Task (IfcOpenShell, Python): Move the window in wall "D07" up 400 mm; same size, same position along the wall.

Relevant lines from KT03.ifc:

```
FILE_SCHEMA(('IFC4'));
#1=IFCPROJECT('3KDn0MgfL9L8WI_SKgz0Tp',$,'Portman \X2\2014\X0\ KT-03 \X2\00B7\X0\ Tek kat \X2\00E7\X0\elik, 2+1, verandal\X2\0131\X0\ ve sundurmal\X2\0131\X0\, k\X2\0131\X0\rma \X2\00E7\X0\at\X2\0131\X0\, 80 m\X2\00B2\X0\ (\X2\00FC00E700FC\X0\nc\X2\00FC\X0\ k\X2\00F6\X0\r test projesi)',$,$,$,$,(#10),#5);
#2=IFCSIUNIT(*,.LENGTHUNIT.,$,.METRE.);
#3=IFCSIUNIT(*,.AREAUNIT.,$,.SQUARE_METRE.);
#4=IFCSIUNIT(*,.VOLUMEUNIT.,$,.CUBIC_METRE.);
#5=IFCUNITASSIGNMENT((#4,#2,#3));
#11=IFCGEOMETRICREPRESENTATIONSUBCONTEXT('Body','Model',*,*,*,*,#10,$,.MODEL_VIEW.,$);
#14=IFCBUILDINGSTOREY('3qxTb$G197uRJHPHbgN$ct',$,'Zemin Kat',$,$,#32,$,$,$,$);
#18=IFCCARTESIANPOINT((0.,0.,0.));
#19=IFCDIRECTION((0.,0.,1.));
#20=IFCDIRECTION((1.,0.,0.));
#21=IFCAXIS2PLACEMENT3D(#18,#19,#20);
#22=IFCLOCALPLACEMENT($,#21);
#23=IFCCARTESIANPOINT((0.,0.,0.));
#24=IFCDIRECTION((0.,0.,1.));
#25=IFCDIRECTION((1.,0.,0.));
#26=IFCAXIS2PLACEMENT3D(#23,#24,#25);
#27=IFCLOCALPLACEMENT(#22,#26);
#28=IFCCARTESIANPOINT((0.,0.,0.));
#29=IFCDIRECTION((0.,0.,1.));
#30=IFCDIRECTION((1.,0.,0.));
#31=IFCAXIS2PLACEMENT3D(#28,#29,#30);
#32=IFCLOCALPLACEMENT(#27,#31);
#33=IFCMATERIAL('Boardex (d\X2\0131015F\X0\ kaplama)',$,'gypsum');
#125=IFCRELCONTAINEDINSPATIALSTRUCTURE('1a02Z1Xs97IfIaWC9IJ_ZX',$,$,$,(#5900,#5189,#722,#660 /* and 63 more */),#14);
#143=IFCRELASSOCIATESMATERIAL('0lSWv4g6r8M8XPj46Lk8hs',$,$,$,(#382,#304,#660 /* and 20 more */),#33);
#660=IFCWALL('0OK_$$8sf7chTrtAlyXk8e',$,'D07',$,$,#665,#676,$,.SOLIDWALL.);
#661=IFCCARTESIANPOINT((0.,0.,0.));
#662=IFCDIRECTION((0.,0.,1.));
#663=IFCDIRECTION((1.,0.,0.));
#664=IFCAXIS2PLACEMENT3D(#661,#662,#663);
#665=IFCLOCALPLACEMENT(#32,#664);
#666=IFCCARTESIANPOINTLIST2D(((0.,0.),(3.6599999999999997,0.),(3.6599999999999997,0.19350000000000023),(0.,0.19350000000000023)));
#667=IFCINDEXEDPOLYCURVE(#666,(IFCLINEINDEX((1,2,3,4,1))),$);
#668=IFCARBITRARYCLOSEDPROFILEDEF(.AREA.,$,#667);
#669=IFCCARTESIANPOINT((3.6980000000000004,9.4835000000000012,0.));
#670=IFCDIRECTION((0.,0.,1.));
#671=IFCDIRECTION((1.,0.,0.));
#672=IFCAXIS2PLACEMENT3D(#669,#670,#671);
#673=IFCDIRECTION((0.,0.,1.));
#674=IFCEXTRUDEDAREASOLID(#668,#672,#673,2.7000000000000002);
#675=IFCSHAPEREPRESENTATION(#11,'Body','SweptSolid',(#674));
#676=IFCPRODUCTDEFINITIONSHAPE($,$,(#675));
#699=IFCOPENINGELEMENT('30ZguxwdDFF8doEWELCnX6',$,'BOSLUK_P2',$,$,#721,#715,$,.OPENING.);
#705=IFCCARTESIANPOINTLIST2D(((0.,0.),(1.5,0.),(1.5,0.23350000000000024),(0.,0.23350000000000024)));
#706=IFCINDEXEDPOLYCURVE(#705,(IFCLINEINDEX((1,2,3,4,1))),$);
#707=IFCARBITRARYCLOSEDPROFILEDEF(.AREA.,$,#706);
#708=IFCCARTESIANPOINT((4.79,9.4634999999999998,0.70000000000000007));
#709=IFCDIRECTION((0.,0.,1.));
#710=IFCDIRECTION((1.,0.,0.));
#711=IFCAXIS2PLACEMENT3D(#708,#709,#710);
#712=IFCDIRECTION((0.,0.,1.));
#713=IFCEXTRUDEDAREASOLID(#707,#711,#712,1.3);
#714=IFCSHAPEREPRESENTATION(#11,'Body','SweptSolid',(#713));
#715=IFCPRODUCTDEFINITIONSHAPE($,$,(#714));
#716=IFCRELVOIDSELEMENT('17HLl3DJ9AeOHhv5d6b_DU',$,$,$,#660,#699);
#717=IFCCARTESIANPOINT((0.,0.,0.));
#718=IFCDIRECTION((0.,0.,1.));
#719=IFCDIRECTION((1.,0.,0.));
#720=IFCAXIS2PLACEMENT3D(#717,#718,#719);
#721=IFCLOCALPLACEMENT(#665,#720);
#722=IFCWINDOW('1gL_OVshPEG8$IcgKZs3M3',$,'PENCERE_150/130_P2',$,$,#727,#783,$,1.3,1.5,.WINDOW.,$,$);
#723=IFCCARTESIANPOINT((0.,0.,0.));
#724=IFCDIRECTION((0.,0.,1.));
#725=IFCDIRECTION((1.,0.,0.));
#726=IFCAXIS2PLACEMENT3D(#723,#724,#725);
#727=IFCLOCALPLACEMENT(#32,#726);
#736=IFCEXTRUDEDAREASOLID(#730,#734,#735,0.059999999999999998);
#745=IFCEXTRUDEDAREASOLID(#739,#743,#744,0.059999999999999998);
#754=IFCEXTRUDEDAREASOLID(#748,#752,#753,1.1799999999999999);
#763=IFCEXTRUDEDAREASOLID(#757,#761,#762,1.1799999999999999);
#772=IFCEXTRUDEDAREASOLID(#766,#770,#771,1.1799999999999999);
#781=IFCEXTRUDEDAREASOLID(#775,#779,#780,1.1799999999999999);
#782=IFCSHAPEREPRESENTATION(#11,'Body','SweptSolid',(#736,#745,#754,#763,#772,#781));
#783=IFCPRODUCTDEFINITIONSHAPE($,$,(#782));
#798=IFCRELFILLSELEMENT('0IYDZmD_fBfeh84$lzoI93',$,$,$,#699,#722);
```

```python
import numpy as np
import ifcopenshell
import ifcopenshell.api.geometry
import ifcopenshell.util.placement
import ifcopenshell.util.unit

model = ifcopenshell.open("KT03.ifc")
unit_scale = ifcopenshell.util.unit.calculate_unit_scale(model)

window = model.by_guid("1gL_OVshPEG8$IcgKZs3M3")
opening = window.FillsVoids[0].RelatingOpeningElement
dz = 0.4 / unit_scale

shift = np.array([0.0, 0.0, dz])
# The window is not placed relative to its opening, so move both.
for product in (opening, window):
    matrix = ifcopenshell.util.placement.get_local_placement(product.ObjectPlacement)
    matrix[:3, 3] += shift
    ifcopenshell.api.geometry.edit_object_placement(model, product=product, matrix=matrix, is_si=False)

print(f"moved by {dz * unit_scale:+.3f} m")

model.write("KT03_edited.ifc")
```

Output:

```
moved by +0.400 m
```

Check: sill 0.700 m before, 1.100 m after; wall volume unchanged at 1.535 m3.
